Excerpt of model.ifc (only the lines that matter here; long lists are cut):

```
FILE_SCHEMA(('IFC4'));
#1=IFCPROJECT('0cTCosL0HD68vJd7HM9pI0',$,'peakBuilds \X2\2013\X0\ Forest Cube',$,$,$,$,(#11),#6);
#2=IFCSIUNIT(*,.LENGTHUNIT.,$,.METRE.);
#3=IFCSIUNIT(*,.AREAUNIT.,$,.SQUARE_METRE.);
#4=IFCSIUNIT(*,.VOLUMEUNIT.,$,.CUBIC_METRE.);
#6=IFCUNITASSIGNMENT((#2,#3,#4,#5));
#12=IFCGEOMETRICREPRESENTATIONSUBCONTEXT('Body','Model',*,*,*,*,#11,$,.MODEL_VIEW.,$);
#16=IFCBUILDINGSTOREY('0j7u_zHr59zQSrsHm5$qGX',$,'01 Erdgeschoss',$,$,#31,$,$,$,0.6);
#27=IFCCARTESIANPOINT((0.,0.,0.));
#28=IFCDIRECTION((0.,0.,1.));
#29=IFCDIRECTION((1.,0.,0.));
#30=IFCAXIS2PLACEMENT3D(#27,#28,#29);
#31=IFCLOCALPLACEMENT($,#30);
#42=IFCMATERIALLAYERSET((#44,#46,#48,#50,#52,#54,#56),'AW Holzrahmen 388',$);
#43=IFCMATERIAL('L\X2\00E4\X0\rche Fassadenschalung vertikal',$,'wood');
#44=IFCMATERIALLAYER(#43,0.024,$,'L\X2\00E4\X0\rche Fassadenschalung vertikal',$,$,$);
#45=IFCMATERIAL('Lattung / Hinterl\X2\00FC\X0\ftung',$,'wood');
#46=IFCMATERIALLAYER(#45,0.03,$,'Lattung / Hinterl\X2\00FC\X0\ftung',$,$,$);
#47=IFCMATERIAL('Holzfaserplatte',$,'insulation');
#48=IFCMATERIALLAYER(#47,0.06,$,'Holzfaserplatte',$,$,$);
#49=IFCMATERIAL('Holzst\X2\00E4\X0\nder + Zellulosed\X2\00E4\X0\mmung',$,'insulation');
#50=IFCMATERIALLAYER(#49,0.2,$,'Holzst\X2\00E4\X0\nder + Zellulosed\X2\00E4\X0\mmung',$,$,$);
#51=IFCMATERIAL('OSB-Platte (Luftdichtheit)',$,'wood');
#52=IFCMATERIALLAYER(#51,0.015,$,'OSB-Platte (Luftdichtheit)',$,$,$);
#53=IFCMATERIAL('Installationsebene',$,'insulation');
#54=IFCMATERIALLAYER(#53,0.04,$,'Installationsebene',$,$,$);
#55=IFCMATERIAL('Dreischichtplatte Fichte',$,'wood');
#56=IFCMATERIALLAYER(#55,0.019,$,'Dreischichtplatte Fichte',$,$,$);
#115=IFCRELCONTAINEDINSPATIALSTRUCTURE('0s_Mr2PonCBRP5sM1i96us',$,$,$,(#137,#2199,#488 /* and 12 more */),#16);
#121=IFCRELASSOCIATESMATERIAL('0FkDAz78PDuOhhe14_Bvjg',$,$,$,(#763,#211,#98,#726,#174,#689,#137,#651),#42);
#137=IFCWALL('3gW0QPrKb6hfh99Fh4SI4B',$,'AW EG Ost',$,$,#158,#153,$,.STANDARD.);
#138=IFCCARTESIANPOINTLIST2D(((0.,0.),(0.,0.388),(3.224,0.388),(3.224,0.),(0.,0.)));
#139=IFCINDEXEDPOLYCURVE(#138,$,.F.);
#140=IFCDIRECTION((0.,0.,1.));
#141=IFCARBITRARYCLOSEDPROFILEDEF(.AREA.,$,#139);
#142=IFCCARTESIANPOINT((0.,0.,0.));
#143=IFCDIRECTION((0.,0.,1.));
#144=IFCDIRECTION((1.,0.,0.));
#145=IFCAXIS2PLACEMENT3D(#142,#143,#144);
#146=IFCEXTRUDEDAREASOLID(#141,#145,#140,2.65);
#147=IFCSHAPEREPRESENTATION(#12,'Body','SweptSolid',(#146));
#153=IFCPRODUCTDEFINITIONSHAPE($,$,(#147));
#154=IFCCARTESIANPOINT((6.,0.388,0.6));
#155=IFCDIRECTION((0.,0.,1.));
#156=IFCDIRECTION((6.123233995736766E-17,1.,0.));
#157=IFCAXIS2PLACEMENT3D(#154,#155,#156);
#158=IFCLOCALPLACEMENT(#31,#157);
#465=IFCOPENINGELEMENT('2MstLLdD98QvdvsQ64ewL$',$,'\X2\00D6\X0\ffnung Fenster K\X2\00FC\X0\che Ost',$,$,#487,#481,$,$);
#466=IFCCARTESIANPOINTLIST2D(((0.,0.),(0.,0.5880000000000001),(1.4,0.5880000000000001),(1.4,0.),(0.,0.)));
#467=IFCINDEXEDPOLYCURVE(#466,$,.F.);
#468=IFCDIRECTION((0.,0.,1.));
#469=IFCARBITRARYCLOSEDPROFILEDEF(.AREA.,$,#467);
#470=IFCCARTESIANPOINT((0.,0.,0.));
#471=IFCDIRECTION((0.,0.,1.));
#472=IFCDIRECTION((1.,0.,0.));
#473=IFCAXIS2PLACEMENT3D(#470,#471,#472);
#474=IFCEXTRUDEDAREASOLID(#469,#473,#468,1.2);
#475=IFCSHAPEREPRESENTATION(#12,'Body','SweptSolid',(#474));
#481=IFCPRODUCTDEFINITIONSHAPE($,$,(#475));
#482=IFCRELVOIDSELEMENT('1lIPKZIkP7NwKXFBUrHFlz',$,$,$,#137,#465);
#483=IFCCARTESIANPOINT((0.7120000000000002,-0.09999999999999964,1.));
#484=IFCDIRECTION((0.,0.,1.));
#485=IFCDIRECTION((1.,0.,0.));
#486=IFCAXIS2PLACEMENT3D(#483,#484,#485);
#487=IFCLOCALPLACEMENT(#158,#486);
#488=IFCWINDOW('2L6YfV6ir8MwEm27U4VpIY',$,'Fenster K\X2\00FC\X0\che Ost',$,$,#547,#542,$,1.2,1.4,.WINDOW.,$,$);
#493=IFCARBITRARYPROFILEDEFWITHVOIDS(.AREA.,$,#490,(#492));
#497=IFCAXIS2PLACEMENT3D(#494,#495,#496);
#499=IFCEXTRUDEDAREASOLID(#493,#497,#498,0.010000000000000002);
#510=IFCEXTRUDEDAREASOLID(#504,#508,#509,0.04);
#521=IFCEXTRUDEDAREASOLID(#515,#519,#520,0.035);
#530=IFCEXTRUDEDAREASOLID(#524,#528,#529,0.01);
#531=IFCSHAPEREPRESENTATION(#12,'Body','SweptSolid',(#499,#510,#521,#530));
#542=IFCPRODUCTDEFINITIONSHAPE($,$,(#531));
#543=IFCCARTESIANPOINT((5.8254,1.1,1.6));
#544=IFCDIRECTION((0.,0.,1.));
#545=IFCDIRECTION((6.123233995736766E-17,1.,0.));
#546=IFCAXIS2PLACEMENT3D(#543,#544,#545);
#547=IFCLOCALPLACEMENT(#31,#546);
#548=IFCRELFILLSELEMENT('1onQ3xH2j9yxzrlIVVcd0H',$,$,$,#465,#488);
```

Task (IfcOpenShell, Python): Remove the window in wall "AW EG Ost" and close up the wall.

```python
import ifcopenshell
import ifcopenshell.api.feature
import ifcopenshell.api.root
import ifcopenshell.geom
import ifcopenshell.util.shape

model = ifcopenshell.open("model.ifc")
settings = ifcopenshell.geom.settings()


def volume(element):
    """Net volume in cubic metres, openings subtracted."""
    shape = ifcopenshell.geom.create_shape(settings, element)
    return ifcopenshell.util.shape.get_volume(shape.geometry)


window = model.by_guid("2L6YfV6ir8MwEm27U4VpIY")
opening = window.FillsVoids[0].RelatingOpeningElement
wall = opening.VoidsElements[0].RelatingBuildingElement
before = volume(wall)

ifcopenshell.api.root.remove_product(model, product=window)
ifcopenshell.api.feature.remove_feature(model, feature=opening)

after = volume(wall)

print(f"wall volume {before:.3f} -> {after:.3f} m3")

model.write("model_updated.ifc")
```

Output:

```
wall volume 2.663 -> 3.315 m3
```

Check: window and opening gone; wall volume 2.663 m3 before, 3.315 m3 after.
